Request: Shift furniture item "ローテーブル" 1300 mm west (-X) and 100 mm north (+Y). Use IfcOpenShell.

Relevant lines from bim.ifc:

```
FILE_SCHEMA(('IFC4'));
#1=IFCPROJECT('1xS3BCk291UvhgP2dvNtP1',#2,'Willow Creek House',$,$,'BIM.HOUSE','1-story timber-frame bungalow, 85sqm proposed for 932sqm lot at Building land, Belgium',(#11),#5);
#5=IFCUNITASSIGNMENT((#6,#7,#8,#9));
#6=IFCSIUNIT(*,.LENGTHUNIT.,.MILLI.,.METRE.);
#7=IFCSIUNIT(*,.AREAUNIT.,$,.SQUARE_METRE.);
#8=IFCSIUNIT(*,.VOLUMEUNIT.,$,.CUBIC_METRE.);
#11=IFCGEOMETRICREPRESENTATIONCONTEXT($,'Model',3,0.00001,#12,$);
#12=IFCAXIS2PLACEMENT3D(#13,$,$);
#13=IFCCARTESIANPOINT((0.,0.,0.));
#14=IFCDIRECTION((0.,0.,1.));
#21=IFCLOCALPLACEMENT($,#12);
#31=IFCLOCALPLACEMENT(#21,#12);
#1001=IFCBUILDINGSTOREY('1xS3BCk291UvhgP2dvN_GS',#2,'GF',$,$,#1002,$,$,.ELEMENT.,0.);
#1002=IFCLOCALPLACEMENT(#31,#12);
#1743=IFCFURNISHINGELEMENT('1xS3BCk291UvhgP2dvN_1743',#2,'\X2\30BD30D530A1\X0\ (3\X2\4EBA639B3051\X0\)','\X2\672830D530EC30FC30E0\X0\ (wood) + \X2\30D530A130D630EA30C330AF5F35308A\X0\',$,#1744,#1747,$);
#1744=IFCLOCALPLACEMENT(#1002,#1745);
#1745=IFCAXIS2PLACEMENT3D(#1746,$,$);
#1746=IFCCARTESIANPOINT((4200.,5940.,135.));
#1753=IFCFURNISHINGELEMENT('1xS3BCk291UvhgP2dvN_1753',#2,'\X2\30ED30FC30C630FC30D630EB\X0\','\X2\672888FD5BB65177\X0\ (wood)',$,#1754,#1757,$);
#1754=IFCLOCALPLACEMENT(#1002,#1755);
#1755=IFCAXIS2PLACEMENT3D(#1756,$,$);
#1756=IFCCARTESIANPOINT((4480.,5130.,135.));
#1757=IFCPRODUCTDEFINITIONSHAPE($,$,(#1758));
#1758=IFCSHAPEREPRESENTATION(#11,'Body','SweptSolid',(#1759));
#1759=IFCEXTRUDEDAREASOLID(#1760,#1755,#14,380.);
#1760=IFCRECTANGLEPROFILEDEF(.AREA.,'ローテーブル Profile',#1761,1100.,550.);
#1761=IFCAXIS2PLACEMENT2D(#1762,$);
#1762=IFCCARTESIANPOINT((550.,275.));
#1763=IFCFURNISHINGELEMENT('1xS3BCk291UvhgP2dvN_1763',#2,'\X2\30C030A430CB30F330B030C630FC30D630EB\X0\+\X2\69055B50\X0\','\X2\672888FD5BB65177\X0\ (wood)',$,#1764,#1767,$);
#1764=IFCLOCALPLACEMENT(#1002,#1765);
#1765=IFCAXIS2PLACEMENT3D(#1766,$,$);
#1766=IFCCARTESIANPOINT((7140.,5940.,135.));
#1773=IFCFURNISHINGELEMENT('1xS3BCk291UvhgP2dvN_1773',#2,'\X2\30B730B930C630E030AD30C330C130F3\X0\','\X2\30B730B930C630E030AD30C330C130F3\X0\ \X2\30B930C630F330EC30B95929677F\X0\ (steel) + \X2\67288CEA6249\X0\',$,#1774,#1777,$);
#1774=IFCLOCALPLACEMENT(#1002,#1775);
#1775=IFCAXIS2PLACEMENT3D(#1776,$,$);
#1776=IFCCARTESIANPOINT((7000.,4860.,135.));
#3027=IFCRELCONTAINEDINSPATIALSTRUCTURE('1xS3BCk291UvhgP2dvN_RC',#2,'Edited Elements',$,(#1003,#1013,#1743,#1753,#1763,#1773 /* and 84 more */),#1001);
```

```python
import ifcopenshell
import ifcopenshell.api.geometry
import ifcopenshell.util.placement

model = ifcopenshell.open("bim.ifc")

item = model.by_guid("1xS3BCk291UvhgP2dvN_1753")
matrix = ifcopenshell.util.placement.get_local_placement(item.ObjectPlacement)
matrix[0, 3] -= 1300.0
matrix[1, 3] += 100.0
ifcopenshell.api.geometry.edit_object_placement(model, product=item, matrix=matrix, is_si=False)

print(ifcopenshell.util.placement.get_local_placement(item.ObjectPlacement).round(3) + 0.0)

model.write("bim_v2.ifc")
```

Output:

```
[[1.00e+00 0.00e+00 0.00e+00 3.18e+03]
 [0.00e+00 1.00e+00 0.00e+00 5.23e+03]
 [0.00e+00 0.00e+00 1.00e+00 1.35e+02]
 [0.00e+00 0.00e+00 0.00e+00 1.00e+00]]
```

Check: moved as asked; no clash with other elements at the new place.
